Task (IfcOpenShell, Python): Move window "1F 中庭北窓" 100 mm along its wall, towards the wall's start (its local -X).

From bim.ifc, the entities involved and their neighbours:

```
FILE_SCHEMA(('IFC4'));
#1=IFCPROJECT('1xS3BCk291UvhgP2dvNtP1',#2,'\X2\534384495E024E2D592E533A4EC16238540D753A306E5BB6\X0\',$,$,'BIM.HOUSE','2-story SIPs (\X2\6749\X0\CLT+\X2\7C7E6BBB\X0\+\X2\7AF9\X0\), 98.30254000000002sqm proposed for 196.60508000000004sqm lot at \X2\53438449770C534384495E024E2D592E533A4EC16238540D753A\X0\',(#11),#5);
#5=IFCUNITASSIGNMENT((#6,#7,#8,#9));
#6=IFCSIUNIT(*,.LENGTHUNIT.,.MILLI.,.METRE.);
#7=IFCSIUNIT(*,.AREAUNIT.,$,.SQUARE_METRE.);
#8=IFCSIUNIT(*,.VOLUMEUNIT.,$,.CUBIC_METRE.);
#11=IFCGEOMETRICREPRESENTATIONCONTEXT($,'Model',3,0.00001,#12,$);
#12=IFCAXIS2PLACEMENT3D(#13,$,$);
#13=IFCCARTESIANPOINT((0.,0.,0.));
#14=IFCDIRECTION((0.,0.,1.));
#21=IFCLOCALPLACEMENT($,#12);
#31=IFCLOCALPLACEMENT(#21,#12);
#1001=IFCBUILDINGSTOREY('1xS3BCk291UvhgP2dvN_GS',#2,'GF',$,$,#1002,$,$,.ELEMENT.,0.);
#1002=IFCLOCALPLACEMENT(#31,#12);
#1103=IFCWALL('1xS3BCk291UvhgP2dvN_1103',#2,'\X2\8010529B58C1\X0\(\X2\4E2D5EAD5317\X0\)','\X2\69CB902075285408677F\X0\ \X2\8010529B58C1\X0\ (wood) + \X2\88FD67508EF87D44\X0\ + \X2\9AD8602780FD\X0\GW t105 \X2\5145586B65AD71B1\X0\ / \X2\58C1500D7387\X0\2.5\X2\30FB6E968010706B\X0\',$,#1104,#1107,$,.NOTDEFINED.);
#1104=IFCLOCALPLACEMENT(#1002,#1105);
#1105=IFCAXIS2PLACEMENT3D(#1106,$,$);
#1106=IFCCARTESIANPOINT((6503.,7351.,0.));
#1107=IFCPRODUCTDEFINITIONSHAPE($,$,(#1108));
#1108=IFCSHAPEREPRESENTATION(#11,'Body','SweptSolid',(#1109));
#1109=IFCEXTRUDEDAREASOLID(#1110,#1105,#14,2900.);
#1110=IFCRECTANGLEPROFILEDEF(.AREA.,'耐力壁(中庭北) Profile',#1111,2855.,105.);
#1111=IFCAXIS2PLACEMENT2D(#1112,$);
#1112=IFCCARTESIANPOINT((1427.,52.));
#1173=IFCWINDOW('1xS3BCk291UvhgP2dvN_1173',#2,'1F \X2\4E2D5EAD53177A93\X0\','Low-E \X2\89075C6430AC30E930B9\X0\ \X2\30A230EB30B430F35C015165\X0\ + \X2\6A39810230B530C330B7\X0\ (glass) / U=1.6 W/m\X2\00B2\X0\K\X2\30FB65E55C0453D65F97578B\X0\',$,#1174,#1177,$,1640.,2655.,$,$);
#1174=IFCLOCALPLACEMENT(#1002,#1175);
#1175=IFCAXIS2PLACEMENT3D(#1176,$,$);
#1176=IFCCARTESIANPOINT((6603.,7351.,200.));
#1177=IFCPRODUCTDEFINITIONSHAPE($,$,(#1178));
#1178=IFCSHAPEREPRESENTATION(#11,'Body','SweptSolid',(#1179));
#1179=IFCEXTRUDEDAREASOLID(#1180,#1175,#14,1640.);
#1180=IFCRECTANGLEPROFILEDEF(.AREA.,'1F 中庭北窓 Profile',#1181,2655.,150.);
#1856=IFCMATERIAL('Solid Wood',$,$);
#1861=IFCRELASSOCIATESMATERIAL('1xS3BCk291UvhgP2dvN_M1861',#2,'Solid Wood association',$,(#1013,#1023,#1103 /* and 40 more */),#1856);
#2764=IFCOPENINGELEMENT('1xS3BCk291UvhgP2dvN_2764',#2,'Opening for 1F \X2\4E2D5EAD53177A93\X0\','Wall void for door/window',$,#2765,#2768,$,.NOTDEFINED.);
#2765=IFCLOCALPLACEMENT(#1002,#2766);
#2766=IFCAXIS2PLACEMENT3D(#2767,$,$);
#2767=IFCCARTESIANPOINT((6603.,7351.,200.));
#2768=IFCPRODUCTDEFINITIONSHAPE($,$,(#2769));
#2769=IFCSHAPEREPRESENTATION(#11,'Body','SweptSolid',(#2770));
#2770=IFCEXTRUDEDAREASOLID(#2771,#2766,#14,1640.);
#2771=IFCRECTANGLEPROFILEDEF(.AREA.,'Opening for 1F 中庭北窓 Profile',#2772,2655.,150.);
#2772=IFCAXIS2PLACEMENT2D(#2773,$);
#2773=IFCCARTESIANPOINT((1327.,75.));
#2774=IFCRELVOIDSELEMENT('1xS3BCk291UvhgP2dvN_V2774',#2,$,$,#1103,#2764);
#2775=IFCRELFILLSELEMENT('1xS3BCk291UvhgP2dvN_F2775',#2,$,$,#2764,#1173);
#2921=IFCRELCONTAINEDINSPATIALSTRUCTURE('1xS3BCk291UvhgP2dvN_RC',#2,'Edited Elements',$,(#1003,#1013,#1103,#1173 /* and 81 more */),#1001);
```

```python
import ifcopenshell
import ifcopenshell.api.geometry
import ifcopenshell.util.placement

model = ifcopenshell.open("bim.ifc")

window = model.by_id(1173)
opening = window.FillsVoids[0].RelatingOpeningElement
wall = opening.VoidsElements[0].RelatingBuildingElement

wall_matrix = ifcopenshell.util.placement.get_local_placement(wall.ObjectPlacement)
shift = wall_matrix[:3, 0] * -100.0
before = ifcopenshell.util.placement.get_local_placement(window.ObjectPlacement)[:3, 3].copy()

# The window is not placed relative to its opening, so move both.
for product in (opening, window):
    matrix = ifcopenshell.util.placement.get_local_placement(product.ObjectPlacement)
    matrix[:3, 3] += shift
    ifcopenshell.api.geometry.edit_object_placement(model, product=product, matrix=matrix, is_si=False)

after = ifcopenshell.util.placement.get_local_placement(window.ObjectPlacement)[:3, 3]
print("window moved by", (after - before).round(3) + 0.0)

model.write("bim_updated.ifc")
```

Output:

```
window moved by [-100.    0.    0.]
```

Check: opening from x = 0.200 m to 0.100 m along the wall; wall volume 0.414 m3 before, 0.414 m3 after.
